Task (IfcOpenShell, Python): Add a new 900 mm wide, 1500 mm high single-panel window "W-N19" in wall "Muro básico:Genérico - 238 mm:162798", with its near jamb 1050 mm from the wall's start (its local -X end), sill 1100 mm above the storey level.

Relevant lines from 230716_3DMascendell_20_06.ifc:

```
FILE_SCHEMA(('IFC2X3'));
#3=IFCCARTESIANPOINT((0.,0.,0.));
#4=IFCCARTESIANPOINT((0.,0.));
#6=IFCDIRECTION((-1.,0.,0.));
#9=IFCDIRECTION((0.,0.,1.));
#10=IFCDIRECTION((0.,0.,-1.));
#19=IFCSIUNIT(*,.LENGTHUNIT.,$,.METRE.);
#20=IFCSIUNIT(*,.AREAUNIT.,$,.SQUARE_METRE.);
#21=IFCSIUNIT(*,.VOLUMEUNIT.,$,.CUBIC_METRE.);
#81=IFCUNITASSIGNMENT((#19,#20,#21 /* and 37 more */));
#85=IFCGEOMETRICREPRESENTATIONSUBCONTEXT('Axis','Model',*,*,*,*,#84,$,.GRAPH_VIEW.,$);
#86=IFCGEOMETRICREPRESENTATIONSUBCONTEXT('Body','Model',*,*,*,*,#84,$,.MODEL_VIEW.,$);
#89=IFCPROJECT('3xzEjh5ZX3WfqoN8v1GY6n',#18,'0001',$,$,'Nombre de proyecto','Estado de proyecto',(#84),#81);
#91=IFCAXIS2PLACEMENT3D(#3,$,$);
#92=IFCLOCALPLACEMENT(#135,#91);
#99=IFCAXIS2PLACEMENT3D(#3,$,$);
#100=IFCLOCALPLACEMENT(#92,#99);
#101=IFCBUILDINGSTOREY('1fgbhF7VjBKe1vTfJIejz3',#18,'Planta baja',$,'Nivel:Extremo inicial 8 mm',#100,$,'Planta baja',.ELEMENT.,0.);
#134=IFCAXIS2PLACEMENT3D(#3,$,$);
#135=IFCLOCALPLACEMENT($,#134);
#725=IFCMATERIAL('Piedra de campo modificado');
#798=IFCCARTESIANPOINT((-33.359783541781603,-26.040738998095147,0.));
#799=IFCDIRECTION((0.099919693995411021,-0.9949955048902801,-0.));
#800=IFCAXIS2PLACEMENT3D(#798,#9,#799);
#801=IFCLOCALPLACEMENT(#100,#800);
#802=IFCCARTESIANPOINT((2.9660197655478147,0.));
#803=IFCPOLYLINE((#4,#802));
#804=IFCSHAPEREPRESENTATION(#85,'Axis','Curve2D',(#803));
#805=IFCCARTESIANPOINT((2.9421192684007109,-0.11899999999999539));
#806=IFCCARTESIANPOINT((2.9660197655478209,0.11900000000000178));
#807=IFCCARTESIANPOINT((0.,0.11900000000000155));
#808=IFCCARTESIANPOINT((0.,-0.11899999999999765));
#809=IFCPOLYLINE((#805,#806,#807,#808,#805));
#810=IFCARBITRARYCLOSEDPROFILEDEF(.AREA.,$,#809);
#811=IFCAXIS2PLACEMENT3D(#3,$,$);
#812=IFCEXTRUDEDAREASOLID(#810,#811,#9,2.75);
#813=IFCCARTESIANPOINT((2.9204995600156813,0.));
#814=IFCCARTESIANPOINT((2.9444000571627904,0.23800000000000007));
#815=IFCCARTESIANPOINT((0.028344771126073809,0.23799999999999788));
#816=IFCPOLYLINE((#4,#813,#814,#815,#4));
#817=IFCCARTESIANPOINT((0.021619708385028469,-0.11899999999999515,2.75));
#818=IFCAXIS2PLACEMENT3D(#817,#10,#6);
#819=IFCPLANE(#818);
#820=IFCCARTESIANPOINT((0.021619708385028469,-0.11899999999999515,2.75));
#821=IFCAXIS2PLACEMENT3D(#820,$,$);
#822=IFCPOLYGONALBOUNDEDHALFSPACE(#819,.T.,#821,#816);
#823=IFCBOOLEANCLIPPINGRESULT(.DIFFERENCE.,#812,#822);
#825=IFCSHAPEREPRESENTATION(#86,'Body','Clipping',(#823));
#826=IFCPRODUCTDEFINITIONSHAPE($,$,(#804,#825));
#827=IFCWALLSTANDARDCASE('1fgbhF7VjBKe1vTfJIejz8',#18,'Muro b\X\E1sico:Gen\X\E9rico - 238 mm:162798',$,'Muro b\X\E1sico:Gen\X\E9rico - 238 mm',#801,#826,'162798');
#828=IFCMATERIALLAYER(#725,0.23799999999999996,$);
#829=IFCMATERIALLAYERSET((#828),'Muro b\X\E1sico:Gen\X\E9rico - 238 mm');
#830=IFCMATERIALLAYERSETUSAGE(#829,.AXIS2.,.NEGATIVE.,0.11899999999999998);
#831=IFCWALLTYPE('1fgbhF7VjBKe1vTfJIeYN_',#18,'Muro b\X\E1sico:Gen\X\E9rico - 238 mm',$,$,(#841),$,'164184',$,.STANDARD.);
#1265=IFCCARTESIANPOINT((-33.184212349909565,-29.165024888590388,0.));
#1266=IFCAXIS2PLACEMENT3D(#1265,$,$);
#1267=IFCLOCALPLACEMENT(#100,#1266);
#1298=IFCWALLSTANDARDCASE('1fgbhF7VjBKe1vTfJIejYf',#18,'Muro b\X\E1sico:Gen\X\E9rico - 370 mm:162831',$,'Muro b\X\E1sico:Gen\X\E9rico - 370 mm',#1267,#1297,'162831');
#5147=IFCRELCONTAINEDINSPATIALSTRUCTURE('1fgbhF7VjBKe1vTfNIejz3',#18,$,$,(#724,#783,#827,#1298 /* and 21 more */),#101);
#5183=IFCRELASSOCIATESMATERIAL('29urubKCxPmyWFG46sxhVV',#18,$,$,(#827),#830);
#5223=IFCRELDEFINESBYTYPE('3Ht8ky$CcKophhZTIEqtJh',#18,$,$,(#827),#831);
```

```python
import numpy as np
import ifcopenshell
import ifcopenshell.api.feature
import ifcopenshell.api.geometry
import ifcopenshell.api.root
import ifcopenshell.api.spatial
import ifcopenshell.api.type
import ifcopenshell.geom
import ifcopenshell.util.element
import ifcopenshell.util.placement
import ifcopenshell.util.representation
import ifcopenshell.util.shape
import ifcopenshell.util.unit

model = ifcopenshell.open("230716_3DMascendell_20_06.ifc")
unit_scale = ifcopenshell.util.unit.calculate_unit_scale(model)
settings = ifcopenshell.geom.settings()


def volume(element):
    """Net volume in cubic metres, openings subtracted."""
    shape = ifcopenshell.geom.create_shape(settings, element)
    return ifcopenshell.util.shape.get_volume(shape.geometry)


wall = model.by_guid("1fgbhF7VjBKe1vTfJIejz8")
storey = ifcopenshell.util.element.get_container(wall, ifc_class="IfcBuildingStorey")
context = ifcopenshell.util.representation.get_context(model, "Model", "Body", "MODEL_VIEW")
before = volume(wall)

width, height, from_end, sill = 0.9, 1.5, 1.05, 1.1  # metres

# The wall runs along its own X axis, and the end named is its -X end.
wall_shape = ifcopenshell.geom.create_shape(settings, wall)
x, y, z = ifcopenshell.util.shape.get_vertices(wall_shape.geometry).T
start = x.min() + from_end
face, thickness = float(y.min()), float(y.max() - y.min())
wall_matrix = ifcopenshell.util.placement.get_local_placement(wall.ObjectPlacement)
level = ifcopenshell.util.placement.get_local_placement(storey.ObjectPlacement)[2, 3]


def in_wall(x, y):
    """Placement at x, y metres in the wall's axes, at sill height."""
    matrix = wall_matrix.copy()
    matrix[:, 3] = wall_matrix @ np.array([x / unit_scale, y / unit_scale, 0.0, 1.0])
    matrix[2, 3] = level + sill / unit_scale
    return matrix


# Opening: a box that overshoots both wall faces by 50 mm.
opening = ifcopenshell.api.root.create_entity(model, ifc_class="IfcOpeningElement")
box = ifcopenshell.api.geometry.add_wall_representation(
    model, context=context, length=width, height=height, thickness=thickness + 0.1
)
ifcopenshell.api.geometry.assign_representation(model, product=opening, representation=box)
ifcopenshell.api.geometry.edit_object_placement(model, product=opening, matrix=in_wall(start, face - 0.05), is_si=False)
ifcopenshell.api.feature.add_feature(model, feature=opening, element=wall)

window = ifcopenshell.api.root.create_entity(model, ifc_class="IfcWindow", name="W-N19")
window.OverallWidth, window.OverallHeight = width / unit_scale, height / unit_scale
body = ifcopenshell.api.geometry.add_window_representation(
    model,
    context=context,
    overall_width=window.OverallWidth,
    overall_height=window.OverallHeight,
    partition_type="SINGLE_PANEL",
)
ifcopenshell.api.geometry.assign_representation(model, product=window, representation=body)
ifcopenshell.api.spatial.assign_container(model, products=[window], relating_structure=storey)
fills = ifcopenshell.api.feature.add_filling(model, opening=opening, element=window)
fills.OwnerHistory = window.OwnerHistory  # required in IFC2X3

# IFC2X3 keeps the operation on the window style.
style = ifcopenshell.api.root.create_entity(model, ifc_class="IfcWindowStyle", name="W-N19")
style.OperationType, style.ConstructionType = "SINGLE_PANEL", "NOTDEFINED"
style.ParameterTakesPrecedence = style.Sizeable = False
ifcopenshell.api.type.assign_type(model, related_objects=[window], relating_type=style)

# Centre the window in the wall's thickness.
ifcopenshell.api.geometry.edit_object_placement(model, product=window, matrix=in_wall(start, face), is_si=False)
window_shape = ifcopenshell.geom.create_shape(settings, window)
depth = ifcopenshell.util.shape.get_vertices(window_shape.geometry)[:, 1]
offset = face + thickness / 2 - (depth.min() + depth.max()) / 2
ifcopenshell.api.geometry.edit_object_placement(model, product=window, matrix=in_wall(start, offset), is_si=False)

after = volume(wall)

print(f"wall volume {before:.3f} -> {after:.3f} m3")

model.write("230716_3DMascendell_20_06_edited.ifc")
```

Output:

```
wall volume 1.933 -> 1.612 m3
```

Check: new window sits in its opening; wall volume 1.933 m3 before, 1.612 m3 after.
